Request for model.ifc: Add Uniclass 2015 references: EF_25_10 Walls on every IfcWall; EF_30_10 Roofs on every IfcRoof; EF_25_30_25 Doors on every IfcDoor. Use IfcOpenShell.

First a look at what the model holds.

```python
import ifcopenshell

model = ifcopenshell.open("model.ifc")
print(model.schema)
print("classifications:", [c.Name for c in model.by_type("IfcClassification")])
for ifc_class in ("IfcDoor", "IfcRoof", "IfcStair", "IfcWall", "IfcWindow"):
    print(ifc_class, len(model.by_type(ifc_class)))
```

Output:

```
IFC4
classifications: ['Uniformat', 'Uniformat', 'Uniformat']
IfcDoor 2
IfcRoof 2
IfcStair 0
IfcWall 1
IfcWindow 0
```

```python
import ifcopenshell
import ifcopenshell.api.classification

model = ifcopenshell.open("model.ifc")

system = ifcopenshell.api.classification.add_classification(model, classification="Uniclass 2015")

codes = {
    "IfcWall": ("EF_25_10", "Walls"),
    "IfcRoof": ("EF_30_10", "Roofs"),
    "IfcDoor": ("EF_25_30_25", "Doors"),
}
for ifc_class, (code, name) in codes.items():
    products = model.by_type(ifc_class)
    ifcopenshell.api.classification.add_reference(
        model, products=products, classification=system, identification=code, name=name
    )
    print(code, len(products))

model.write("model_updated.ifc")
```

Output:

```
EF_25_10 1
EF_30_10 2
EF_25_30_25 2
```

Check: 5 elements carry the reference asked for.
